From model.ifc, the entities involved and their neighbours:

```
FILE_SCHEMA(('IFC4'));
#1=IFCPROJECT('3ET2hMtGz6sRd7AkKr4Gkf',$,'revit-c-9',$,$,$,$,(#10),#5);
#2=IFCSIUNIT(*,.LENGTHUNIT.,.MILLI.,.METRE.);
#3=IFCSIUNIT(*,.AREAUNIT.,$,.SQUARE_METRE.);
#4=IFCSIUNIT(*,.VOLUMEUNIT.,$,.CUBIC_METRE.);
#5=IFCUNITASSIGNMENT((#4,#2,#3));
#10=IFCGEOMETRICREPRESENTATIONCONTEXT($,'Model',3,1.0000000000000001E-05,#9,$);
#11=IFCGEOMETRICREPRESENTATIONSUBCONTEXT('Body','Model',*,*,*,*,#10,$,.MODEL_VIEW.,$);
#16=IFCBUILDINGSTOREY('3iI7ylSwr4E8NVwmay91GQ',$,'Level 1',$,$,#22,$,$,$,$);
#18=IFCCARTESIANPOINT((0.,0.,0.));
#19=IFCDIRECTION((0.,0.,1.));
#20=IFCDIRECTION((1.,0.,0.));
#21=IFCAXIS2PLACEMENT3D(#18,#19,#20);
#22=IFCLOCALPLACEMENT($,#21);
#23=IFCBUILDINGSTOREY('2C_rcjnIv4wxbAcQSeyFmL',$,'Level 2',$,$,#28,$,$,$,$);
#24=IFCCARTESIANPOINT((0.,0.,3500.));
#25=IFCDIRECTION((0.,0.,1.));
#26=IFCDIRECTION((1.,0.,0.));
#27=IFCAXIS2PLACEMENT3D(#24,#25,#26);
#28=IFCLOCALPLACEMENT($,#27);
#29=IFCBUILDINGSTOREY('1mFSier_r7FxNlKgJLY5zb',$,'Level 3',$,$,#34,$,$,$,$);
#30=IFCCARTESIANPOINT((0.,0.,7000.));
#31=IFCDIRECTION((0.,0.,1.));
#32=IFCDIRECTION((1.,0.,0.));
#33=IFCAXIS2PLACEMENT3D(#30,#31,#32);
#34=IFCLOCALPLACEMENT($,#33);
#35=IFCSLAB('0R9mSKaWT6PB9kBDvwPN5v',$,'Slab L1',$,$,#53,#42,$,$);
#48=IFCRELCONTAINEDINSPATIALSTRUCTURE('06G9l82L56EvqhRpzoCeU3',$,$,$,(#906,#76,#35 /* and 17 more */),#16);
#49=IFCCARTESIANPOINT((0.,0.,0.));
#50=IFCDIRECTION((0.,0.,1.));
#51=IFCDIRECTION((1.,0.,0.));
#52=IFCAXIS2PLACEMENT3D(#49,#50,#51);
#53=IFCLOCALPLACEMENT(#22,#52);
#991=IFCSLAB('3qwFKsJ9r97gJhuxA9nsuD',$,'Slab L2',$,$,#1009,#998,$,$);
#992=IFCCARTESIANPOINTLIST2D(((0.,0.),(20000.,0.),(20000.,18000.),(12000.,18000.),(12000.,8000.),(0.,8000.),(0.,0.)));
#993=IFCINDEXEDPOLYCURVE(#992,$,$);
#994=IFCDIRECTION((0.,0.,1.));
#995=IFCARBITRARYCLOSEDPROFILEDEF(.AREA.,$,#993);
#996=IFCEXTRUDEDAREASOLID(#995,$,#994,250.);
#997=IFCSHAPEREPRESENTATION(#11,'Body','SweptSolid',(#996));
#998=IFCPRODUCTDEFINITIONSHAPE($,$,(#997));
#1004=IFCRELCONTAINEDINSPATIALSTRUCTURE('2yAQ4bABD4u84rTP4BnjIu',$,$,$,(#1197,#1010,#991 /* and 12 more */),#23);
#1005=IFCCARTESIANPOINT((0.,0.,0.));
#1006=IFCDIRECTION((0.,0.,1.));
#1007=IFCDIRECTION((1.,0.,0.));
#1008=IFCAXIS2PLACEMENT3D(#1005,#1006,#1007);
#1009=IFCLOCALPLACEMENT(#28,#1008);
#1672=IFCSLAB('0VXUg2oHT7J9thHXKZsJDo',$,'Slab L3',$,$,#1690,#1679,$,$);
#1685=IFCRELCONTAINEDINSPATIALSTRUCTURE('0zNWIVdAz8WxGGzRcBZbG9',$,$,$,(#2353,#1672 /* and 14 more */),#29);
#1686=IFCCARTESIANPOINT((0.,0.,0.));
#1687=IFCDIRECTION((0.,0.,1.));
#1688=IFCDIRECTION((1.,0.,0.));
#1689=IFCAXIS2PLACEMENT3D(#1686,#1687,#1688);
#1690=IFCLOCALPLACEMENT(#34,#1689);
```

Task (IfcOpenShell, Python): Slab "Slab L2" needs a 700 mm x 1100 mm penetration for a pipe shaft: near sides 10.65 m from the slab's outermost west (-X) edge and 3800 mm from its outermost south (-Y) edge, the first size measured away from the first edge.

```python
import numpy as np
import ifcopenshell
import ifcopenshell.api.feature
import ifcopenshell.api.geometry
import ifcopenshell.api.root
import ifcopenshell.geom
import ifcopenshell.util.placement
import ifcopenshell.util.representation
import ifcopenshell.util.shape
import ifcopenshell.util.unit

model = ifcopenshell.open("model.ifc")
unit_scale = ifcopenshell.util.unit.calculate_unit_scale(model)
settings = ifcopenshell.geom.settings()


def volume(element):
    """Net volume in cubic metres, openings subtracted."""
    shape = ifcopenshell.geom.create_shape(settings, element)
    return ifcopenshell.util.shape.get_volume(shape.geometry)


slab = model.by_id(991)
before = volume(slab)

# Extent in the slab's own axes, in metres. The edges named are its -X and -Y sides.
slab_shape = ifcopenshell.geom.create_shape(settings, slab)
vertices = ifcopenshell.util.shape.get_vertices(slab_shape.geometry)
x_min, y_min, bottom = vertices.min(axis=0)
top = vertices[:, 2].max()

opening = ifcopenshell.api.root.create_entity(model, ifc_class="IfcOpeningElement", name="Pipe shaft opening", predefined_type="OPENING")
context = ifcopenshell.util.representation.get_context(model, "Model", "Body", "MODEL_VIEW")
width, depth = 0.7, 1.1
outline = [(0.0, 0.0), (width, 0.0), (width, depth), (0.0, depth), (0.0, 0.0)]
# Overshoot both faces by 50 mm so the cut is clean.
shape = ifcopenshell.api.geometry.add_slab_representation(
    model, context=context, depth=top - bottom + 0.1, polyline=outline
)
ifcopenshell.api.geometry.assign_representation(model, product=opening, representation=shape)

matrix = ifcopenshell.util.placement.get_local_placement(slab.ObjectPlacement)
matrix[:, 3] = matrix @ np.append(np.array([x_min + 10.65, y_min + 3.8, bottom - 0.05]) / unit_scale, 1.0)
ifcopenshell.api.geometry.edit_object_placement(model, product=opening, matrix=matrix, is_si=False)
ifcopenshell.api.feature.add_feature(model, feature=opening, element=slab)

after = volume(slab)

print(f"slab volume {before:.3f} -> {after:.3f} m3")

model.write("model_v2.ifc")
```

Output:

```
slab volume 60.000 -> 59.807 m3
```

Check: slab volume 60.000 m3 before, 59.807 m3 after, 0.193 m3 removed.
